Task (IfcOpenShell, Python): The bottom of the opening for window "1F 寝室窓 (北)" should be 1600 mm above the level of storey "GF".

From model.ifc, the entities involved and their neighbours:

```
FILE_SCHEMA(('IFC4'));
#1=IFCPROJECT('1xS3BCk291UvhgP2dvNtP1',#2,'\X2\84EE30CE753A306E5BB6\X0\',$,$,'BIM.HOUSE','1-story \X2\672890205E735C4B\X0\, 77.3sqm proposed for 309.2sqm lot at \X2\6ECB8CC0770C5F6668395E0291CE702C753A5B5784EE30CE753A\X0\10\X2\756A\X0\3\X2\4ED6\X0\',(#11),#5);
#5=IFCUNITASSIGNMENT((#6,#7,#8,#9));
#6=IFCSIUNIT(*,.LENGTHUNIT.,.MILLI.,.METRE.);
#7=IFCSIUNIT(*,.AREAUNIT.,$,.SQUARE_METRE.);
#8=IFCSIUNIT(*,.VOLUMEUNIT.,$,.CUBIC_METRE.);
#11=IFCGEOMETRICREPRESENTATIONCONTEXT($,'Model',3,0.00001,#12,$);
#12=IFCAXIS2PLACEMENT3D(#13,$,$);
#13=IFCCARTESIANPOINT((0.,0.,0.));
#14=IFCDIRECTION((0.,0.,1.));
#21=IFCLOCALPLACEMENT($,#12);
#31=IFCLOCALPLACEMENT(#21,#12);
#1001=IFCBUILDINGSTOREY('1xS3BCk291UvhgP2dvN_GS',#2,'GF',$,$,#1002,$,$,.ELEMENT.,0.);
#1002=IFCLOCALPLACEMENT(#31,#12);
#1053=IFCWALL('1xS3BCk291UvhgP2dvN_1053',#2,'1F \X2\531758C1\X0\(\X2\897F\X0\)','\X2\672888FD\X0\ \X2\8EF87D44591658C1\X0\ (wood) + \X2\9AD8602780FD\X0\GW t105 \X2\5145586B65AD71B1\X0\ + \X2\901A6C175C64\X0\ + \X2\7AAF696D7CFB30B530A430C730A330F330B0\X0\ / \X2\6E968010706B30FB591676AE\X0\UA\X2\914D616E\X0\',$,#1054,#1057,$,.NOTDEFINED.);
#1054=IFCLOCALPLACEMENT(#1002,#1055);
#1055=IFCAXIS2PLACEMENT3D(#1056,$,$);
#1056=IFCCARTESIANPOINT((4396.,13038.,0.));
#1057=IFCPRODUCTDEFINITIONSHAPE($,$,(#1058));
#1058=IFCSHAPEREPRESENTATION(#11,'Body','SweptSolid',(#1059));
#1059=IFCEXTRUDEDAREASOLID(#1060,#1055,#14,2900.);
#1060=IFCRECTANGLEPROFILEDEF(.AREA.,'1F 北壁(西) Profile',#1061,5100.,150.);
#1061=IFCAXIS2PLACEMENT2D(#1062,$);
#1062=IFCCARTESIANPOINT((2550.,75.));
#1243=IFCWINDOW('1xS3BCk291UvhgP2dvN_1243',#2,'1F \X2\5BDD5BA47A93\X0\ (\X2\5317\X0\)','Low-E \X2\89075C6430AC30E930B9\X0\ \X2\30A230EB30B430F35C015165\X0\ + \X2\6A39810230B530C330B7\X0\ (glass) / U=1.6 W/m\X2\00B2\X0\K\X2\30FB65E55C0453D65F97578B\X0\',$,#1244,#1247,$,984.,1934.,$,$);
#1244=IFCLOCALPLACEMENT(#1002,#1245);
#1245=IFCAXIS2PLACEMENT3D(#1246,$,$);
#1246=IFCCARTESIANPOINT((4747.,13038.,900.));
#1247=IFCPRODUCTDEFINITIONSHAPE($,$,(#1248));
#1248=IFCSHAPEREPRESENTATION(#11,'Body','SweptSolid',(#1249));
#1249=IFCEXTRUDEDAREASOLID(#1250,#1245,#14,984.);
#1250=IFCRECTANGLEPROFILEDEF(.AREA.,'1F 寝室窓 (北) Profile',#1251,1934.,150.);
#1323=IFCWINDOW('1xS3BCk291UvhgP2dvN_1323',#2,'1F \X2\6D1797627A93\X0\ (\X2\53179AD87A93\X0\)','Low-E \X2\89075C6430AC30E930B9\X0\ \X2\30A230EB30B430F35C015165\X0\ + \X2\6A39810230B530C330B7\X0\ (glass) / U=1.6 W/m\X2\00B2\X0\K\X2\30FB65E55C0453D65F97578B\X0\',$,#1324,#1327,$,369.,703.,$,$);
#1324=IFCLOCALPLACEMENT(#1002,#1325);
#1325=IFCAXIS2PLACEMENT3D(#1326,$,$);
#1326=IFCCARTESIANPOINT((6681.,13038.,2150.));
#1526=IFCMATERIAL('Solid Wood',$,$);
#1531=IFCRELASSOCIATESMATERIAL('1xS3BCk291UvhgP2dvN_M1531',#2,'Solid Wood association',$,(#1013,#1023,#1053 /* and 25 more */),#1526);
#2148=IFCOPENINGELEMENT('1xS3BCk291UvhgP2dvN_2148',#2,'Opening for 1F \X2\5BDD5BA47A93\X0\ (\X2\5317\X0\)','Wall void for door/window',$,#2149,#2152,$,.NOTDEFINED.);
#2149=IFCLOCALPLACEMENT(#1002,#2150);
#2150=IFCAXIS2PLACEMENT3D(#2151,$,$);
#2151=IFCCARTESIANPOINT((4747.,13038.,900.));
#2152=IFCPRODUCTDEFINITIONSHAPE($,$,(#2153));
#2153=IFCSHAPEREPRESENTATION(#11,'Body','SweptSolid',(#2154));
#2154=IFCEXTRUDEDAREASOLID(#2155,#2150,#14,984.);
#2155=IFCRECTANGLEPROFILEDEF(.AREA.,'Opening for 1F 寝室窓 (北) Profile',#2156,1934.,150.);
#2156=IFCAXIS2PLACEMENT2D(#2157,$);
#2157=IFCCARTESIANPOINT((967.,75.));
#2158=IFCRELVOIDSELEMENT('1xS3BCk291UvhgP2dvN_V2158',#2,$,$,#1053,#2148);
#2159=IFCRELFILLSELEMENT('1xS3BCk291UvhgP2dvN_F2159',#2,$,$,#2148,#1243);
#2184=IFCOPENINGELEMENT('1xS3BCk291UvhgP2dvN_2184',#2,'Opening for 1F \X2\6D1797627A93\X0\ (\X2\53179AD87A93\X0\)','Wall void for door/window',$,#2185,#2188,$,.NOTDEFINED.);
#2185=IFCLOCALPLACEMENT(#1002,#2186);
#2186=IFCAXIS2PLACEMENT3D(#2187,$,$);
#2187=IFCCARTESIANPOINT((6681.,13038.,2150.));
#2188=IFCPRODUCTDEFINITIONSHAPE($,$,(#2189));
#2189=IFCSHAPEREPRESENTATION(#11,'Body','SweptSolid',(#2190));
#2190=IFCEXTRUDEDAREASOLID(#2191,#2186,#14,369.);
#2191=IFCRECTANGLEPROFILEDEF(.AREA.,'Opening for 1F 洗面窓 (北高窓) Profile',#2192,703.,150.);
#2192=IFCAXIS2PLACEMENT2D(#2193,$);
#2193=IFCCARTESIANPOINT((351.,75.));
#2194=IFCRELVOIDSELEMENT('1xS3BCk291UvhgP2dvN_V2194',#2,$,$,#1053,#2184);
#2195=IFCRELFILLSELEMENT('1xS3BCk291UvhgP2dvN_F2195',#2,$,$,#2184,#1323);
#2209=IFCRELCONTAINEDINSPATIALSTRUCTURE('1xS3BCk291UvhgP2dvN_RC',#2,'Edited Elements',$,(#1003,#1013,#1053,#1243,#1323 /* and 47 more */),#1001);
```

```python
import numpy as np
import ifcopenshell
import ifcopenshell.api.geometry
import ifcopenshell.geom
import ifcopenshell.util.element
import ifcopenshell.util.placement
import ifcopenshell.util.shape
import ifcopenshell.util.unit

model = ifcopenshell.open("model.ifc")
unit_scale = ifcopenshell.util.unit.calculate_unit_scale(model)

window = model.by_guid("1xS3BCk291UvhgP2dvN_1243")
opening = window.FillsVoids[0].RelatingOpeningElement
storey = ifcopenshell.util.element.get_container(window, ifc_class="IfcBuildingStorey")
level = ifcopenshell.util.placement.get_local_placement(storey.ObjectPlacement)[2, 3]

# The opening's origin need not be at the sill, so measure its lowest point.
shape = ifcopenshell.geom.create_shape(ifcopenshell.geom.settings(), opening)
bottom = ifcopenshell.util.shape.get_shape_bottom_elevation(shape, shape.geometry) / unit_scale
dz = level + 1600.0 - bottom

shift = np.array([0.0, 0.0, dz])
# The window is not placed relative to its opening, so move both.
for product in (opening, window):
    matrix = ifcopenshell.util.placement.get_local_placement(product.ObjectPlacement)
    matrix[:3, 3] += shift
    ifcopenshell.api.geometry.edit_object_placement(model, product=product, matrix=matrix, is_si=False)

print(f"moved by {dz * unit_scale:+.3f} m")

model.write("model_v2.ifc")
```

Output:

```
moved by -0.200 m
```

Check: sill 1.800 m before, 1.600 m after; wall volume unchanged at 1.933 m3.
